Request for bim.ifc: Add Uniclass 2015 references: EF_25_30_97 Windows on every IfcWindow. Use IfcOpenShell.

First a look at what the model holds.

```python
import ifcopenshell

model = ifcopenshell.open("bim.ifc")
print(model.schema)
print("classifications:", [c.Name for c in model.by_type("IfcClassification")])
for ifc_class in ("IfcDoor", "IfcRoof", "IfcStair", "IfcWall", "IfcWindow"):
    print(ifc_class, len(model.by_type(ifc_class)))
```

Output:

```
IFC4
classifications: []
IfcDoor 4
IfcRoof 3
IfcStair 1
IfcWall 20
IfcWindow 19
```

```python
import ifcopenshell
import ifcopenshell.api.classification

model = ifcopenshell.open("bim.ifc")

system = ifcopenshell.api.classification.add_classification(model, classification="Uniclass 2015")

codes = {
    "IfcWindow": ("EF_25_30_97", "Windows"),
}
for ifc_class, (code, name) in codes.items():
    products = model.by_type(ifc_class)
    ifcopenshell.api.classification.add_reference(
        model, products=products, classification=system, identification=code, name=name
    )
    print(code, len(products))

model.write("bim_updated.ifc")
```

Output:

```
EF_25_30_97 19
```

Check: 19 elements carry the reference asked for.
